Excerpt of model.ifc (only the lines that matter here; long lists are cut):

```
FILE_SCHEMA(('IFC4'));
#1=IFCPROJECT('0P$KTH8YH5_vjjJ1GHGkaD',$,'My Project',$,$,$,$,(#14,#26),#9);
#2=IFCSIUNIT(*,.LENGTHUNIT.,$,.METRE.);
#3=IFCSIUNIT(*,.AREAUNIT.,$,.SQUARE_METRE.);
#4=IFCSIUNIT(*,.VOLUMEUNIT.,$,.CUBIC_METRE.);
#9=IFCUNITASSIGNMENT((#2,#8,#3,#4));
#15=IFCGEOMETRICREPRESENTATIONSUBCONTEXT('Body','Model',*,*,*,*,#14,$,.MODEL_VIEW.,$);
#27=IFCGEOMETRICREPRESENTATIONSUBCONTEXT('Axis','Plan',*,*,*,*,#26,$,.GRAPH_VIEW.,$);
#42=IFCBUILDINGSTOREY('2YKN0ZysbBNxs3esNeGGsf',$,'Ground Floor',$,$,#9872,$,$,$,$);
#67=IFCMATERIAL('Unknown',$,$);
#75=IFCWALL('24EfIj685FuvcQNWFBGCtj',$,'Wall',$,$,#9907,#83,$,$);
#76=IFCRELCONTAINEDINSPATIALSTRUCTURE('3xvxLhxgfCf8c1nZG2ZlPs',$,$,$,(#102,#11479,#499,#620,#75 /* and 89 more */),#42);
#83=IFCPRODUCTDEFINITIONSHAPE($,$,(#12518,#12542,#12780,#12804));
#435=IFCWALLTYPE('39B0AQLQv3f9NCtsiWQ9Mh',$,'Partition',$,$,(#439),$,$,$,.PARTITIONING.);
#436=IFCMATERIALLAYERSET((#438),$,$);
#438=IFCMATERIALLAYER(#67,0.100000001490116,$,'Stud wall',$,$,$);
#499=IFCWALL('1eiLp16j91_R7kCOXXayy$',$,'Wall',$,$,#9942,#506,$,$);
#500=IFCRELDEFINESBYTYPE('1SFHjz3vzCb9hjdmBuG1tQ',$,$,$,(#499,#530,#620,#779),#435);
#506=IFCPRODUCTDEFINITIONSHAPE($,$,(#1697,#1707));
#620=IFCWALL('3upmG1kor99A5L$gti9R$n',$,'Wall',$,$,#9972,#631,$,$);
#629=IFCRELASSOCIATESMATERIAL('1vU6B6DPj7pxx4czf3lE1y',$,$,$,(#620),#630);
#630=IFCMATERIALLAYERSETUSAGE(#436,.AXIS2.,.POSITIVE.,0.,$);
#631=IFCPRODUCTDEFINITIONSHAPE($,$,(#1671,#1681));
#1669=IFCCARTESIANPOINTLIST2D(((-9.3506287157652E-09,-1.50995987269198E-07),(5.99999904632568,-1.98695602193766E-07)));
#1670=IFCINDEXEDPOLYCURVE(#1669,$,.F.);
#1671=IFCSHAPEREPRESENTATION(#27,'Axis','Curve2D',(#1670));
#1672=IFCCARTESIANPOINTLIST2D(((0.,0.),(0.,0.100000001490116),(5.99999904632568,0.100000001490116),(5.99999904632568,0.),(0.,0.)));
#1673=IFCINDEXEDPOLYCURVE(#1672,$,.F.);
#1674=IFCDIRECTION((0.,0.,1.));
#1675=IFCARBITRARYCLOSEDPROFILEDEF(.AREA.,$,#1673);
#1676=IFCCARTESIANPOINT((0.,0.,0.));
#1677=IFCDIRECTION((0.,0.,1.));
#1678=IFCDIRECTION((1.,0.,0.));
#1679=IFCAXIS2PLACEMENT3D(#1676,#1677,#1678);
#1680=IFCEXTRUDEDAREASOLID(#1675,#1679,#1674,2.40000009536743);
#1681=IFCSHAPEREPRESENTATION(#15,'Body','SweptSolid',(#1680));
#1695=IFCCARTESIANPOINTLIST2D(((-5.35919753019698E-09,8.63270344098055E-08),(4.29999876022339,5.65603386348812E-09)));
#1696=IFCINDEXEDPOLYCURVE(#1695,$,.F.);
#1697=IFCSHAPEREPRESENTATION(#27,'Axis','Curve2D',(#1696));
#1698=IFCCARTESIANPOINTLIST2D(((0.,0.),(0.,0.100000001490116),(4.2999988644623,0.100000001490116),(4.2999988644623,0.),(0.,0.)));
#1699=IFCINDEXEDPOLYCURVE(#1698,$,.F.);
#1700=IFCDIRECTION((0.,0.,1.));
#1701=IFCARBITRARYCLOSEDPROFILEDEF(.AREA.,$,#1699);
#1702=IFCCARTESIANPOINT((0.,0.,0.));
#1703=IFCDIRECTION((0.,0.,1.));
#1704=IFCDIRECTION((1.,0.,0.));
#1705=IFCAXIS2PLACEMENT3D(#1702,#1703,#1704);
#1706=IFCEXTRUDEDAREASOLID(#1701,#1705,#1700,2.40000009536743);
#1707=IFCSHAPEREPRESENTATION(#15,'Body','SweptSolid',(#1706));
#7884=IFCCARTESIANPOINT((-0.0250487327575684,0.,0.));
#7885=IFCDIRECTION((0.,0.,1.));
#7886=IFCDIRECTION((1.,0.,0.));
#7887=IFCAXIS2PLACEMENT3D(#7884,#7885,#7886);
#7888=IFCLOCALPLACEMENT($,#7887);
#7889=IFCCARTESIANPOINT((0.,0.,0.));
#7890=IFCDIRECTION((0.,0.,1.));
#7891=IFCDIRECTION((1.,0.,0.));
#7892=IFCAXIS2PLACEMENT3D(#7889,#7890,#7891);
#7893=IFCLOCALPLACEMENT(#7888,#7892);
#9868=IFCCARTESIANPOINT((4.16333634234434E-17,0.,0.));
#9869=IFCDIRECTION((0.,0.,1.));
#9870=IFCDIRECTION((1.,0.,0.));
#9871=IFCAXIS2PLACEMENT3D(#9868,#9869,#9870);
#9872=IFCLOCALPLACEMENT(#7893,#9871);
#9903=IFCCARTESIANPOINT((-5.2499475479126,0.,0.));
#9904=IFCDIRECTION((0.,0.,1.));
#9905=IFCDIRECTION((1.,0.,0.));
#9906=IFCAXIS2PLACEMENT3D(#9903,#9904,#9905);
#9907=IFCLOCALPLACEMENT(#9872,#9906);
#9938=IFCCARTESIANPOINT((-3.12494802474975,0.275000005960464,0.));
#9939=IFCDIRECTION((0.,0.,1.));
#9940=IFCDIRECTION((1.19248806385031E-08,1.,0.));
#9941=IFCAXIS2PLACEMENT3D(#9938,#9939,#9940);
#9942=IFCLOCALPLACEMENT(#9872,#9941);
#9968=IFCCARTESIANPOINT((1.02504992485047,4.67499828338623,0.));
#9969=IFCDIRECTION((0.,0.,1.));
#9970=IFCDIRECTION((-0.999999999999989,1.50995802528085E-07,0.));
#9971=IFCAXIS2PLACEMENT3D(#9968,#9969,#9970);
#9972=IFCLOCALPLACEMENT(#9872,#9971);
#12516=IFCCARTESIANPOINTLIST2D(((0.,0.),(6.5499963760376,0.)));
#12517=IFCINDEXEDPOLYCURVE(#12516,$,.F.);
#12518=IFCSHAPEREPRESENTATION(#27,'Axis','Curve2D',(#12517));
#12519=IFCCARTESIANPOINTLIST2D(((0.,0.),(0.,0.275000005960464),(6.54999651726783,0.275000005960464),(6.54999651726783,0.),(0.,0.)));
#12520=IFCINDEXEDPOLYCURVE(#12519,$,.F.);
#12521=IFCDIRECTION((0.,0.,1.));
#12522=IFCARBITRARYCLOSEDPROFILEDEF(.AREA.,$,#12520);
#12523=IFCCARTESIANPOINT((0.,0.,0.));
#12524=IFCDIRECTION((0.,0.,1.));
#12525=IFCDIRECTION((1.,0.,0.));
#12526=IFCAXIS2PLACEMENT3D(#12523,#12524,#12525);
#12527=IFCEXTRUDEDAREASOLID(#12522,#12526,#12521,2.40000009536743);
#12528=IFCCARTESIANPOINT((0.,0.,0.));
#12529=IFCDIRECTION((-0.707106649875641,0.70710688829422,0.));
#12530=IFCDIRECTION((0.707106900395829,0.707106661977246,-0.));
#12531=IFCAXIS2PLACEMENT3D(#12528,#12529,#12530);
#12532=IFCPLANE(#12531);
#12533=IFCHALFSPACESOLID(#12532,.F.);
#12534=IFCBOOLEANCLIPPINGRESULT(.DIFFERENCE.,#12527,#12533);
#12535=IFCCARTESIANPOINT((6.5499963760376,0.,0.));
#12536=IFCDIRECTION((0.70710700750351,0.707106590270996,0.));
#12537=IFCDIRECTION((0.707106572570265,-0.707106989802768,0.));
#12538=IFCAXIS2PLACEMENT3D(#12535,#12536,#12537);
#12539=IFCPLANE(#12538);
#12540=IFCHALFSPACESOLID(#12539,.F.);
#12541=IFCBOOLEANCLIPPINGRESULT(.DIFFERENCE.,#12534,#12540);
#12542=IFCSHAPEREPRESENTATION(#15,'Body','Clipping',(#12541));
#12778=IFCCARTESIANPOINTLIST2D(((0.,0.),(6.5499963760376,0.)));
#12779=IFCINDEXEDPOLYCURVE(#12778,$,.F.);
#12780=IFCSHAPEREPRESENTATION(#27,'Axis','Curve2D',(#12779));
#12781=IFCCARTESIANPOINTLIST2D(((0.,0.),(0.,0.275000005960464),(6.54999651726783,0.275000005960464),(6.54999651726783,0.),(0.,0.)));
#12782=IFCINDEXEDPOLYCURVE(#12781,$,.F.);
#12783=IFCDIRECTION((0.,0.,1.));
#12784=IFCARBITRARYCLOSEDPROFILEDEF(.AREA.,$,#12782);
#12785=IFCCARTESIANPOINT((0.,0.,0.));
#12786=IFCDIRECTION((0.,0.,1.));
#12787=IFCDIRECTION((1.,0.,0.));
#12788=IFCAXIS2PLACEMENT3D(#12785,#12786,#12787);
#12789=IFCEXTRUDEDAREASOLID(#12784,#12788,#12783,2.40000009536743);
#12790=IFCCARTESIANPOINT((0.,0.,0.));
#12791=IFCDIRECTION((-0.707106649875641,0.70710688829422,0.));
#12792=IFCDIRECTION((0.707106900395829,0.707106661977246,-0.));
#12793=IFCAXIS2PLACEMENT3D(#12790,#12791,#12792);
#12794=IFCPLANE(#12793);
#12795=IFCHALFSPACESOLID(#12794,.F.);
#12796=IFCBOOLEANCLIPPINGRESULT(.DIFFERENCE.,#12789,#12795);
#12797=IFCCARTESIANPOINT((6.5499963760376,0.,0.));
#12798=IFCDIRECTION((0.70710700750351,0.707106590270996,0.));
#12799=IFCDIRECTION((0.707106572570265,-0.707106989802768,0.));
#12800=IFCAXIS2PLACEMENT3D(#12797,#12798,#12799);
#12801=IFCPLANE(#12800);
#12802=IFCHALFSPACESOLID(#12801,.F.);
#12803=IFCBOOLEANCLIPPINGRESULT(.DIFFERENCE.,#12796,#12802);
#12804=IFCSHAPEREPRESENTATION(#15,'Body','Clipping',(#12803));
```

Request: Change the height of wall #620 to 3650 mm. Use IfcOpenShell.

```python
import ifcopenshell
import ifcopenshell.geom
import ifcopenshell.util.representation
import ifcopenshell.util.shape
import ifcopenshell.util.unit

model = ifcopenshell.open("model.ifc")
unit_scale = ifcopenshell.util.unit.calculate_unit_scale(model)
settings = ifcopenshell.geom.settings()


def volume(element):
    """Net volume in cubic metres, openings subtracted."""
    shape = ifcopenshell.geom.create_shape(settings, element)
    return ifcopenshell.util.shape.get_volume(shape.geometry)


wall = model.by_guid("3upmG1kor99A5L$gti9R$n")
before = volume(wall)

body = ifcopenshell.util.representation.get_representation(wall, "Model", "Body")
solid = body.Items[0]
old_height = solid.Depth
solid.Depth = 3.65 / unit_scale
after = volume(wall)

print(f"height {old_height:g} -> {solid.Depth:g}, volume {before:.3f} -> {after:.3f} m3")

model.write("model_rev.ifc")
```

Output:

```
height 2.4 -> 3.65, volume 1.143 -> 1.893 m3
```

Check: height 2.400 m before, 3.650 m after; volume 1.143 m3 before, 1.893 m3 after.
